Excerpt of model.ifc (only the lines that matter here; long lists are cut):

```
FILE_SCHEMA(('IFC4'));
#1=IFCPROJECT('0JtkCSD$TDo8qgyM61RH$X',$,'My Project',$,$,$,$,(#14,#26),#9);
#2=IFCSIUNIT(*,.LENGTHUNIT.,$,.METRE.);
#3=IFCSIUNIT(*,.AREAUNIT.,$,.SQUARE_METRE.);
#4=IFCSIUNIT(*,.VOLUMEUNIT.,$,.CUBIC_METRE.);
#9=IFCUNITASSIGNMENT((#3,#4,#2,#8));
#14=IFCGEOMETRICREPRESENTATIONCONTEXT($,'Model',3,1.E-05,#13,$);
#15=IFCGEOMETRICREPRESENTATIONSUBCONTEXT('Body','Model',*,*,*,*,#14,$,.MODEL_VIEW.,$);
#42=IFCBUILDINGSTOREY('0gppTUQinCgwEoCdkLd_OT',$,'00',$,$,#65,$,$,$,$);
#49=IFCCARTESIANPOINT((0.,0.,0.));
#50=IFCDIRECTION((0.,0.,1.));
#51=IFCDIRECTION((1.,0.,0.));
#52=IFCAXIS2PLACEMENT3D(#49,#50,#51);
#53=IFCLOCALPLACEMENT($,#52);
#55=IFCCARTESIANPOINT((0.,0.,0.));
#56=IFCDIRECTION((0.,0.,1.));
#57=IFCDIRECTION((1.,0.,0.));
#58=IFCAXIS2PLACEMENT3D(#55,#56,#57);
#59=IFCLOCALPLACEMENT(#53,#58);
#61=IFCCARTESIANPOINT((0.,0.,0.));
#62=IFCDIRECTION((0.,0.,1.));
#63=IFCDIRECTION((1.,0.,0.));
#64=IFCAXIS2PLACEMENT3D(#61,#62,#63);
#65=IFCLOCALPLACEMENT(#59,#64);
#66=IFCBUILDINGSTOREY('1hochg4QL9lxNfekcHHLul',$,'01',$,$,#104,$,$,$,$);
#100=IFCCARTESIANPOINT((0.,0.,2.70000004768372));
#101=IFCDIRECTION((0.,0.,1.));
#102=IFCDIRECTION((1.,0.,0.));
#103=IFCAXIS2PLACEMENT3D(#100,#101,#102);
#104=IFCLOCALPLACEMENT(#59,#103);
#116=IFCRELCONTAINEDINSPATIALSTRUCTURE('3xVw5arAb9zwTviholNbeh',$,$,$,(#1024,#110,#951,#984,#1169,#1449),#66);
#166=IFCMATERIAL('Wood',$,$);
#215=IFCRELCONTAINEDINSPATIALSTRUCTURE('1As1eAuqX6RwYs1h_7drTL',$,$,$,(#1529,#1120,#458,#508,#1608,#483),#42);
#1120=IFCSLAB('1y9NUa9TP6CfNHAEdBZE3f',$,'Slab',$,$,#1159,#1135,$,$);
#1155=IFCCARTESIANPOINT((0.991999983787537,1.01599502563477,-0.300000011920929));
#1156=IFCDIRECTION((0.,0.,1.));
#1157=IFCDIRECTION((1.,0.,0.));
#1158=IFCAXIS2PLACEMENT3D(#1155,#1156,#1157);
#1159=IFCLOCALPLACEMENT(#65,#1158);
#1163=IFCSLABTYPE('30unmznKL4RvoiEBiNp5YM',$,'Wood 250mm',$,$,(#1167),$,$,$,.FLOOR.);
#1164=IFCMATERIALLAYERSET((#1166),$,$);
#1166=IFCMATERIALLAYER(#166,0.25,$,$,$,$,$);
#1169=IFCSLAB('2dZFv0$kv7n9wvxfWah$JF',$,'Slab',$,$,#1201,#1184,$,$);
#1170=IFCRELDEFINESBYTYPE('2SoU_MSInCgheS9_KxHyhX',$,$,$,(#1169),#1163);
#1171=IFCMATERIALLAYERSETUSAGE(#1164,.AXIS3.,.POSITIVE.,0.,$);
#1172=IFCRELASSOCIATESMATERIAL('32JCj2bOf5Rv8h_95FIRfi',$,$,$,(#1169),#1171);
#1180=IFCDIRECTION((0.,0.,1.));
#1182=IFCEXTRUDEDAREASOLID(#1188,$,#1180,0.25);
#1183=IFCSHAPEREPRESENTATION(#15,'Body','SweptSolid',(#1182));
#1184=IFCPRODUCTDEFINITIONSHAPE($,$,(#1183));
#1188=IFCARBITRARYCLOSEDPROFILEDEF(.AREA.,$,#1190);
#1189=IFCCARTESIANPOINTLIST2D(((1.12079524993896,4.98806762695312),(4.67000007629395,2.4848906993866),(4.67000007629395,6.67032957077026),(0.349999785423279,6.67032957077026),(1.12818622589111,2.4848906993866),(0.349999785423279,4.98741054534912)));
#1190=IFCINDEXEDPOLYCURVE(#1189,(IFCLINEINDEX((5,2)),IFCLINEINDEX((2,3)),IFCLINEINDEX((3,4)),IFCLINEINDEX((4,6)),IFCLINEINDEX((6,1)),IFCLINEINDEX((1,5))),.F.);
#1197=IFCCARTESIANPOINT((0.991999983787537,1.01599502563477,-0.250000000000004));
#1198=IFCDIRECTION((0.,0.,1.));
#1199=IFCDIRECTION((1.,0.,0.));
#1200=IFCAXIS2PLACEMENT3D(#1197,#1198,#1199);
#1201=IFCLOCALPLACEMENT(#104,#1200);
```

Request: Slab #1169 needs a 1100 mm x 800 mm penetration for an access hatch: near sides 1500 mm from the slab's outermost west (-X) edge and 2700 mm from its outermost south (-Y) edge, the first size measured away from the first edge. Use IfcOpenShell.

```python
import numpy as np
import ifcopenshell
import ifcopenshell.api.feature
import ifcopenshell.api.geometry
import ifcopenshell.api.root
import ifcopenshell.geom
import ifcopenshell.util.placement
import ifcopenshell.util.representation
import ifcopenshell.util.shape
import ifcopenshell.util.unit

model = ifcopenshell.open("model.ifc")
unit_scale = ifcopenshell.util.unit.calculate_unit_scale(model)
settings = ifcopenshell.geom.settings()


def volume(element):
    """Net volume in cubic metres, openings subtracted."""
    shape = ifcopenshell.geom.create_shape(settings, element)
    return ifcopenshell.util.shape.get_volume(shape.geometry)


slab = model.by_guid("2dZFv0$kv7n9wvxfWah$JF")
before = volume(slab)

# Extent in the slab's own axes, in metres. The edges named are its -X and -Y sides.
slab_shape = ifcopenshell.geom.create_shape(settings, slab)
vertices = ifcopenshell.util.shape.get_vertices(slab_shape.geometry)
x_min, y_min, bottom = vertices.min(axis=0)
top = vertices[:, 2].max()

opening = ifcopenshell.api.root.create_entity(model, ifc_class="IfcOpeningElement", name="Access hatch opening", predefined_type="OPENING")
context = ifcopenshell.util.representation.get_context(model, "Model", "Body", "MODEL_VIEW")
width, depth = 1.1, 0.8
outline = [(0.0, 0.0), (width, 0.0), (width, depth), (0.0, depth), (0.0, 0.0)]
# Overshoot both faces by 50 mm so the cut is clean.
shape = ifcopenshell.api.geometry.add_slab_representation(
    model, context=context, depth=top - bottom + 0.1, polyline=outline
)
ifcopenshell.api.geometry.assign_representation(model, product=opening, representation=shape)

matrix = ifcopenshell.util.placement.get_local_placement(slab.ObjectPlacement)
matrix[:, 3] = matrix @ np.append(np.array([x_min + 1.5, y_min + 2.7, bottom - 0.05]) / unit_scale, 1.0)
ifcopenshell.api.geometry.edit_object_placement(model, product=opening, matrix=matrix, is_si=False)
ifcopenshell.api.feature.add_feature(model, feature=opening, element=slab)

after = volume(slab)

print(f"slab volume {before:.3f} -> {after:.3f} m3")

model.write("model_rev.ifc")
```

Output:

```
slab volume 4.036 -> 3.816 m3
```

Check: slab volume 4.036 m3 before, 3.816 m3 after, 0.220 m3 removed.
